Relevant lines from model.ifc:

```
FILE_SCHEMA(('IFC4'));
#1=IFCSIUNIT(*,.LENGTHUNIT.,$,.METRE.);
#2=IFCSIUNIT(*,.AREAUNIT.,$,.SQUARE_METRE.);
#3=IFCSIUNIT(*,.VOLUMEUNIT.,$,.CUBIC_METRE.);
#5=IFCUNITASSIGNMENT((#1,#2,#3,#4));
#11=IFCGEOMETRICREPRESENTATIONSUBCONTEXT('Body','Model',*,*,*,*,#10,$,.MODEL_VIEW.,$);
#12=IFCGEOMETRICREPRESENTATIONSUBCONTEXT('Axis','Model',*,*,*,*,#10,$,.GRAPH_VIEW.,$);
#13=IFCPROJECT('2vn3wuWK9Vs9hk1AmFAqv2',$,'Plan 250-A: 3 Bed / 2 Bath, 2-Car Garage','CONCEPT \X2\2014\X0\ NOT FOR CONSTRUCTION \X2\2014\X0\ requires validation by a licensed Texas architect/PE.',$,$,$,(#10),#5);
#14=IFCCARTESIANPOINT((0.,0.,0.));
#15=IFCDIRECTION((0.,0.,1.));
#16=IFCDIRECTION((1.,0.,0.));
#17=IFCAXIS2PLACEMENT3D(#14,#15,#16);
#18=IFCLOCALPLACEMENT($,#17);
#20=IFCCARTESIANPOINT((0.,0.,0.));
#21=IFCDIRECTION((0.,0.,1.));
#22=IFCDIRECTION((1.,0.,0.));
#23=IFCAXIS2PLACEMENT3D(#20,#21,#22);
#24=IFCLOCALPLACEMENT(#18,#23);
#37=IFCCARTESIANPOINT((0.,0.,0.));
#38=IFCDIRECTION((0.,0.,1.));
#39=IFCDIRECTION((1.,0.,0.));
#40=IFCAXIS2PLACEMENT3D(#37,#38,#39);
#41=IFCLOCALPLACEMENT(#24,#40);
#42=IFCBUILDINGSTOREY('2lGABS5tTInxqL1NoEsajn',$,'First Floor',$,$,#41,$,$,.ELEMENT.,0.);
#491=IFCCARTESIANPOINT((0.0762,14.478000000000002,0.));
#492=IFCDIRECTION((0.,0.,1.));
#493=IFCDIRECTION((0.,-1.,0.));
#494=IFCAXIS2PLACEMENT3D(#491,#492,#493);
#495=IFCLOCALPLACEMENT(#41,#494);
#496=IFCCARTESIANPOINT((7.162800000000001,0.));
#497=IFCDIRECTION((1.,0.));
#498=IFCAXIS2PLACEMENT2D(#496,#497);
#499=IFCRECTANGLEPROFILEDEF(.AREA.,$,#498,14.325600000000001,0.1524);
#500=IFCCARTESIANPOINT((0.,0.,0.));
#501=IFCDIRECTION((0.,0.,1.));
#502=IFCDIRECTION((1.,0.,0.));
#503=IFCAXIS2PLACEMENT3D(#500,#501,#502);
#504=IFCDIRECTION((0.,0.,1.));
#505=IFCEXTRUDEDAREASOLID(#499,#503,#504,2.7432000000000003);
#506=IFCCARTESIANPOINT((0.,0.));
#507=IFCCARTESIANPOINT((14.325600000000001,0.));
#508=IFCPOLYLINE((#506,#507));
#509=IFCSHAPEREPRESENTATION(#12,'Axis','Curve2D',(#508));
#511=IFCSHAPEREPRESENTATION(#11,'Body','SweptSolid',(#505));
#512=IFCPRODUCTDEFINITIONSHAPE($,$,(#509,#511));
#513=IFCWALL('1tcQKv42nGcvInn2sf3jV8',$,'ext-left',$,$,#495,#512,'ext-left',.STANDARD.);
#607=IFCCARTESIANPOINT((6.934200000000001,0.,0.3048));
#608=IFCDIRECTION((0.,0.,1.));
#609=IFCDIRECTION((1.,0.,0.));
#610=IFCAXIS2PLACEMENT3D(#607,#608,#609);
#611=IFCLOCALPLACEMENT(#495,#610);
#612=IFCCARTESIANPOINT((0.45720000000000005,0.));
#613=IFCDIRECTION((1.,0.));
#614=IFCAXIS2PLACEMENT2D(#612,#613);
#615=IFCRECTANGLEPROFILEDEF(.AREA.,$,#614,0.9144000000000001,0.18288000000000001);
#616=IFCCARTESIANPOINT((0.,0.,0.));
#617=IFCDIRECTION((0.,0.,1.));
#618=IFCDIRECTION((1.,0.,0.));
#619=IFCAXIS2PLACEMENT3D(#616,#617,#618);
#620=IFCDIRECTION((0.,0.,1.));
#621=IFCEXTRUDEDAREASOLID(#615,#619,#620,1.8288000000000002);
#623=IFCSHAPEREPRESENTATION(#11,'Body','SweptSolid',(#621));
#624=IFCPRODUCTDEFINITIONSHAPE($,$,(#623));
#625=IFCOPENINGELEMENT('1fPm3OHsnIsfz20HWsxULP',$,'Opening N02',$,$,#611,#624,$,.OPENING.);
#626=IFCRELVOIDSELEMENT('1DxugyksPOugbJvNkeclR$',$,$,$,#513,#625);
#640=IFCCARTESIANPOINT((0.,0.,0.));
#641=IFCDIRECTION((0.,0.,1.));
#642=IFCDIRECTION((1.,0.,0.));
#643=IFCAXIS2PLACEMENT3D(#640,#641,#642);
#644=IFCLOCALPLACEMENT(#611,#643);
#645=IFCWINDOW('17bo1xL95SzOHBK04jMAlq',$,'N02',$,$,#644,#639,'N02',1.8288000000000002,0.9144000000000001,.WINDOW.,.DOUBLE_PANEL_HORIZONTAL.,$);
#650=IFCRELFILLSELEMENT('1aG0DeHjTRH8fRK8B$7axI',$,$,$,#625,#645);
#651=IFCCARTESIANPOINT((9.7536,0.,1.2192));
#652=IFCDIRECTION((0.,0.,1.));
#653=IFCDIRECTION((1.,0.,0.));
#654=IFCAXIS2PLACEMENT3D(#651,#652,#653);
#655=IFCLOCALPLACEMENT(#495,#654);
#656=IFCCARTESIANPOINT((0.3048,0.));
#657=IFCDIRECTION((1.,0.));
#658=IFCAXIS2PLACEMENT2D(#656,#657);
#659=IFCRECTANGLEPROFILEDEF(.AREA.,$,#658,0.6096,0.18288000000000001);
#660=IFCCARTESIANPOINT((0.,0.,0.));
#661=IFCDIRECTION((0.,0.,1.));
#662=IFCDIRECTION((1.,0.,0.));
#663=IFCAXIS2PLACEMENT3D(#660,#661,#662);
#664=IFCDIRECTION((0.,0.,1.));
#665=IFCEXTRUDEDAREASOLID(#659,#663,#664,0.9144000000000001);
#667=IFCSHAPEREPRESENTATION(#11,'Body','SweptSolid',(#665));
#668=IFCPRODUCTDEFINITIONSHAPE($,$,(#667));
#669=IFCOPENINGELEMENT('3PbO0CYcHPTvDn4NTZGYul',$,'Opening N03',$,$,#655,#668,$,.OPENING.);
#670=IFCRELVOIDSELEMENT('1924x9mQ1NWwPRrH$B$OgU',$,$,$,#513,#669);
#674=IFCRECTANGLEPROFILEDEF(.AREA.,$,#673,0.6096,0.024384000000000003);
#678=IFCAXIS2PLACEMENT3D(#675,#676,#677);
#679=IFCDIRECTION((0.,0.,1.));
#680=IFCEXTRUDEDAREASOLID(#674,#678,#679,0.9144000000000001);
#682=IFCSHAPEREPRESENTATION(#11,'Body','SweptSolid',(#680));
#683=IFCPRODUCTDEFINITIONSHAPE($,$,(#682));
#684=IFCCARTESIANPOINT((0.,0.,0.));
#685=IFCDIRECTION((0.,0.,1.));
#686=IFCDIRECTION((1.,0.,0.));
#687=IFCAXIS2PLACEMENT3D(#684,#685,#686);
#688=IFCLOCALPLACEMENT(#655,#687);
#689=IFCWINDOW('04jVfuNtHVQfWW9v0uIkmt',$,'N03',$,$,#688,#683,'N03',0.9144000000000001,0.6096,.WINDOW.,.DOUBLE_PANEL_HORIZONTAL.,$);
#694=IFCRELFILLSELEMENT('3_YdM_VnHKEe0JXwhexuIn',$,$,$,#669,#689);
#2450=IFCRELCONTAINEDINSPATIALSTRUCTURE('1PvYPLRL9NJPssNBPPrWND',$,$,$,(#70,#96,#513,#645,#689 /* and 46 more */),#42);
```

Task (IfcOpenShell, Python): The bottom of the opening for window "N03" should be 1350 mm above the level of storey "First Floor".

```python
import numpy as np
import ifcopenshell
import ifcopenshell.api.geometry
import ifcopenshell.geom
import ifcopenshell.util.element
import ifcopenshell.util.placement
import ifcopenshell.util.shape
import ifcopenshell.util.unit

model = ifcopenshell.open("model.ifc")
unit_scale = ifcopenshell.util.unit.calculate_unit_scale(model)

window = model.by_guid("04jVfuNtHVQfWW9v0uIkmt")
opening = window.FillsVoids[0].RelatingOpeningElement
storey = ifcopenshell.util.element.get_container(window, ifc_class="IfcBuildingStorey")
level = ifcopenshell.util.placement.get_local_placement(storey.ObjectPlacement)[2, 3]

# The opening's origin need not be at the sill, so measure its lowest point.
shape = ifcopenshell.geom.create_shape(ifcopenshell.geom.settings(), opening)
bottom = ifcopenshell.util.shape.get_shape_bottom_elevation(shape, shape.geometry) / unit_scale
dz = level + 1.35 - bottom

shift = np.array([0.0, 0.0, dz])
# The window is placed relative to its opening, so it follows when the opening moves.
matrix = ifcopenshell.util.placement.get_local_placement(opening.ObjectPlacement)
matrix[:3, 3] += shift
ifcopenshell.api.geometry.edit_object_placement(
    model, product=opening, matrix=matrix, is_si=False, should_transform_children=True
)

print(f"moved by {dz * unit_scale:+.3f} m")

model.write("model-out.ifc")
```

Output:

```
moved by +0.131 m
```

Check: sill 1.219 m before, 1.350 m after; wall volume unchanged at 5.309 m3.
